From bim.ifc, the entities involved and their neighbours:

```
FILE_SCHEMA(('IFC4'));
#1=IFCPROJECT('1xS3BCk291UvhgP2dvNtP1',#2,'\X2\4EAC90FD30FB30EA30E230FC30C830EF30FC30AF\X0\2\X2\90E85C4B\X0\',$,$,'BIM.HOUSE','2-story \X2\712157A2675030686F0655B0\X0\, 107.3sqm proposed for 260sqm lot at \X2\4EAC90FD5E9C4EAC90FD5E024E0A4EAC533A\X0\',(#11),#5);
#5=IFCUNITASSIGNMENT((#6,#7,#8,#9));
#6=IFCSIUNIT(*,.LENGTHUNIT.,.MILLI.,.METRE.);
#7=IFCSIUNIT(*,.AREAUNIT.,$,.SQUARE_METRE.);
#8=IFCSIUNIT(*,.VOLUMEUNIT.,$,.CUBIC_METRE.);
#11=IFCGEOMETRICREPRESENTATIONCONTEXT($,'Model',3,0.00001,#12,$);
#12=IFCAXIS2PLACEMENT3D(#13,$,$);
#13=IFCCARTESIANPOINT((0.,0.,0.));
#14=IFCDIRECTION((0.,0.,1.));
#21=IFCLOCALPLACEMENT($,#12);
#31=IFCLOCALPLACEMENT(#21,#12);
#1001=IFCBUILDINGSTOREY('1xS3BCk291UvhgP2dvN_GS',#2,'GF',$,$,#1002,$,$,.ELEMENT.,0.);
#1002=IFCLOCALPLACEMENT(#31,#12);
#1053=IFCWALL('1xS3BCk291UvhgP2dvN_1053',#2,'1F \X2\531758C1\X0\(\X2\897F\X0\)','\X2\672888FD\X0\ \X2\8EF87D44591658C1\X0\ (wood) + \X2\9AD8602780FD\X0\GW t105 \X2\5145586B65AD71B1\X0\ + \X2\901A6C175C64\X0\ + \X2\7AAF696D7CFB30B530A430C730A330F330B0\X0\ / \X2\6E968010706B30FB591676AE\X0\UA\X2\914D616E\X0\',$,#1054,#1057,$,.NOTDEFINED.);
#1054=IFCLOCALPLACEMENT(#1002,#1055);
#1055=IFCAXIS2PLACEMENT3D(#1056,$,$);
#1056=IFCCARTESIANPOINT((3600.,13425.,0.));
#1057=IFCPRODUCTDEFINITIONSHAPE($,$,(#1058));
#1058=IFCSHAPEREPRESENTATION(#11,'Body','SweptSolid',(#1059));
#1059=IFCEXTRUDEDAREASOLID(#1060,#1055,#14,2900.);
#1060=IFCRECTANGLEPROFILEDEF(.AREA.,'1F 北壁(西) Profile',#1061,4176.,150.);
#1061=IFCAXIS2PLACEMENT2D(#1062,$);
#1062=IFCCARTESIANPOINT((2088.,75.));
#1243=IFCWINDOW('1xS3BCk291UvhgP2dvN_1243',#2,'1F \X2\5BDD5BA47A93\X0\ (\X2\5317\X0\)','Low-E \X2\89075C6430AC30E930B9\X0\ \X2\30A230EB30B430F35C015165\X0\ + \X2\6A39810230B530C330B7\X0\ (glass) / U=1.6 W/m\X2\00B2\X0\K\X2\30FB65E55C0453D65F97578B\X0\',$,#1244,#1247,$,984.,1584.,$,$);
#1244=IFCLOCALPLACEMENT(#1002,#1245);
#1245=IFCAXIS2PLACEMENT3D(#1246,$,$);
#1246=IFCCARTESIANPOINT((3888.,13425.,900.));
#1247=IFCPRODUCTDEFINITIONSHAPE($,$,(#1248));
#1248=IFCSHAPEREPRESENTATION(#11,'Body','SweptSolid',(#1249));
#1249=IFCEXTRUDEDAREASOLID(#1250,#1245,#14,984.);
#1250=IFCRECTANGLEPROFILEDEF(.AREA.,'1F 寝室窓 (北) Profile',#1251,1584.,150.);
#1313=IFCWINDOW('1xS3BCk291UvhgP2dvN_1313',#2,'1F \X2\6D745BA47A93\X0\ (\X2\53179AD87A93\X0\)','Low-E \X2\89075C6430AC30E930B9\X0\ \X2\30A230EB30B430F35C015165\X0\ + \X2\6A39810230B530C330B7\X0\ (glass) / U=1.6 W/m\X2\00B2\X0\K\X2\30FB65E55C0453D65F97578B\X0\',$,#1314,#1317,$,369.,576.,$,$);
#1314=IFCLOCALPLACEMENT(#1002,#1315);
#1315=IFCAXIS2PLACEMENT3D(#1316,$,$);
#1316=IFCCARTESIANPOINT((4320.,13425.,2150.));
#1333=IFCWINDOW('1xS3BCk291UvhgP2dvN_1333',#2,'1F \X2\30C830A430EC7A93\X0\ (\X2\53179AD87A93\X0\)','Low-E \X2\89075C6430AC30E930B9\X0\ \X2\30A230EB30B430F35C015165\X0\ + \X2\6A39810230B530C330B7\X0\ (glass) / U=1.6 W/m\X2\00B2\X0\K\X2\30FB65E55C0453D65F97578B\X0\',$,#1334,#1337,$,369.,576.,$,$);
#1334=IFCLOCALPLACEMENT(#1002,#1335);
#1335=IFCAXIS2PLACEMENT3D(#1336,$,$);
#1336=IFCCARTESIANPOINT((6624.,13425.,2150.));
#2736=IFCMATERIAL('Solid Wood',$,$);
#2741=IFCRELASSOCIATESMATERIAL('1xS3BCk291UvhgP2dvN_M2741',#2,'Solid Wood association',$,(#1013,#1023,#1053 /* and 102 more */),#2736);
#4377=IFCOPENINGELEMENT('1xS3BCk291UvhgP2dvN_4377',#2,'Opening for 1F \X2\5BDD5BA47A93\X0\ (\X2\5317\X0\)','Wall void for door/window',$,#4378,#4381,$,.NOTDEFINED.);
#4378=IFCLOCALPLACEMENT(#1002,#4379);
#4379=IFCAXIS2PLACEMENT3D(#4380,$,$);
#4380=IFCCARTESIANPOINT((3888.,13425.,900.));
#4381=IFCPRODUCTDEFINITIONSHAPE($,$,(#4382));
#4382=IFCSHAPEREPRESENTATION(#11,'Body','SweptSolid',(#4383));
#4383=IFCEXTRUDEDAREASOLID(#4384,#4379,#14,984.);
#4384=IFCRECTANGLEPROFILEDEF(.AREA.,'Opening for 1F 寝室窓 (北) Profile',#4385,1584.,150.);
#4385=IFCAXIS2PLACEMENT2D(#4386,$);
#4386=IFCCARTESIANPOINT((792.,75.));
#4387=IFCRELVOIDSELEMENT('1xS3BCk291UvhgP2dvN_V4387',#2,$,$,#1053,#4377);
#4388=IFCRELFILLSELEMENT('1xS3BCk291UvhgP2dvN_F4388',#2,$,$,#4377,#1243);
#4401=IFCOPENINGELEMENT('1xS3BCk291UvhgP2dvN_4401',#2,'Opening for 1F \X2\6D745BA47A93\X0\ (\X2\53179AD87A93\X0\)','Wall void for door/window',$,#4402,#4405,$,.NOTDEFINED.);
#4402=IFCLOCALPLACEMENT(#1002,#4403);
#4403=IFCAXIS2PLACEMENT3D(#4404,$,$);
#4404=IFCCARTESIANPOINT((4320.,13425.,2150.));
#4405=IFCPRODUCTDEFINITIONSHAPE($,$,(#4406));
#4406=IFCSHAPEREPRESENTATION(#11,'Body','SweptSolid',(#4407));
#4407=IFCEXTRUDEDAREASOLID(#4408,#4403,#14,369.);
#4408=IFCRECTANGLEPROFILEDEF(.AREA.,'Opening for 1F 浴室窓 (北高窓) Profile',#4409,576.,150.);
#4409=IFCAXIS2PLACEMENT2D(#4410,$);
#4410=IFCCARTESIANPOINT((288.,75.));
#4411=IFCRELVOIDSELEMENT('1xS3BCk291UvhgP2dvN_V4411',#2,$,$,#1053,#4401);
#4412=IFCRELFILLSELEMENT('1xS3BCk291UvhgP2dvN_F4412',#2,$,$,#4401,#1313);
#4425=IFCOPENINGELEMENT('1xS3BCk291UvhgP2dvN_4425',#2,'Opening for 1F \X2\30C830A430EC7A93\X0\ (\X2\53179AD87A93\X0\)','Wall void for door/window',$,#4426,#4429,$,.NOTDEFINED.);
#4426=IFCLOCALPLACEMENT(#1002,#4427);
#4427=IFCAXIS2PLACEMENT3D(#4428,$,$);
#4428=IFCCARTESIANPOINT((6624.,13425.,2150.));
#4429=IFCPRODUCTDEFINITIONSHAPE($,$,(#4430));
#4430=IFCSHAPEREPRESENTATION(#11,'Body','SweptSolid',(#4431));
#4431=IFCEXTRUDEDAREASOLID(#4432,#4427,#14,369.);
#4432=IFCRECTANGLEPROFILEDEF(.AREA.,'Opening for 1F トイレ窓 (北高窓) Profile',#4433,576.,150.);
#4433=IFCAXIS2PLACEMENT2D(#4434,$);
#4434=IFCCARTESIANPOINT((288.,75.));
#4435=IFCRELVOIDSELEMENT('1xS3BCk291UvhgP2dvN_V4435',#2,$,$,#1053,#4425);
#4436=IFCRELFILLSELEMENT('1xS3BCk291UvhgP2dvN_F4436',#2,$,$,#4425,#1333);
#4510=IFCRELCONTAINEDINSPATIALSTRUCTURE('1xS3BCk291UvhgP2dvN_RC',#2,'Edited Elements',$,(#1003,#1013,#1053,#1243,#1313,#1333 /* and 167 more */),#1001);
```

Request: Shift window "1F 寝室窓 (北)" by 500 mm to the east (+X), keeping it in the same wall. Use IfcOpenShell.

```python
import ifcopenshell
import ifcopenshell.api.geometry
import ifcopenshell.util.placement
import ifcopenshell.util.unit

model = ifcopenshell.open("bim.ifc")
unit_scale = ifcopenshell.util.unit.calculate_unit_scale(model)

window = model.by_guid("1xS3BCk291UvhgP2dvN_1243")
opening = window.FillsVoids[0].RelatingOpeningElement
wall = opening.VoidsElements[0].RelatingBuildingElement

wall_matrix = ifcopenshell.util.placement.get_local_placement(wall.ObjectPlacement)
shift = wall_matrix[:3, 0] * 0.5 / unit_scale
before = ifcopenshell.util.placement.get_local_placement(window.ObjectPlacement)[:3, 3].copy()

# The window is not placed relative to its opening, so move both.
for product in (opening, window):
    matrix = ifcopenshell.util.placement.get_local_placement(product.ObjectPlacement)
    matrix[:3, 3] += shift
    ifcopenshell.api.geometry.edit_object_placement(model, product=product, matrix=matrix, is_si=False)

after = ifcopenshell.util.placement.get_local_placement(window.ObjectPlacement)[:3, 3]
print("window moved by", (after - before).round(3) + 0.0)

model.write("bim_edited.ifc")
```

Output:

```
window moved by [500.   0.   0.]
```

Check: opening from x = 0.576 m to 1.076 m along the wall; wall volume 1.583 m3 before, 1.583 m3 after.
